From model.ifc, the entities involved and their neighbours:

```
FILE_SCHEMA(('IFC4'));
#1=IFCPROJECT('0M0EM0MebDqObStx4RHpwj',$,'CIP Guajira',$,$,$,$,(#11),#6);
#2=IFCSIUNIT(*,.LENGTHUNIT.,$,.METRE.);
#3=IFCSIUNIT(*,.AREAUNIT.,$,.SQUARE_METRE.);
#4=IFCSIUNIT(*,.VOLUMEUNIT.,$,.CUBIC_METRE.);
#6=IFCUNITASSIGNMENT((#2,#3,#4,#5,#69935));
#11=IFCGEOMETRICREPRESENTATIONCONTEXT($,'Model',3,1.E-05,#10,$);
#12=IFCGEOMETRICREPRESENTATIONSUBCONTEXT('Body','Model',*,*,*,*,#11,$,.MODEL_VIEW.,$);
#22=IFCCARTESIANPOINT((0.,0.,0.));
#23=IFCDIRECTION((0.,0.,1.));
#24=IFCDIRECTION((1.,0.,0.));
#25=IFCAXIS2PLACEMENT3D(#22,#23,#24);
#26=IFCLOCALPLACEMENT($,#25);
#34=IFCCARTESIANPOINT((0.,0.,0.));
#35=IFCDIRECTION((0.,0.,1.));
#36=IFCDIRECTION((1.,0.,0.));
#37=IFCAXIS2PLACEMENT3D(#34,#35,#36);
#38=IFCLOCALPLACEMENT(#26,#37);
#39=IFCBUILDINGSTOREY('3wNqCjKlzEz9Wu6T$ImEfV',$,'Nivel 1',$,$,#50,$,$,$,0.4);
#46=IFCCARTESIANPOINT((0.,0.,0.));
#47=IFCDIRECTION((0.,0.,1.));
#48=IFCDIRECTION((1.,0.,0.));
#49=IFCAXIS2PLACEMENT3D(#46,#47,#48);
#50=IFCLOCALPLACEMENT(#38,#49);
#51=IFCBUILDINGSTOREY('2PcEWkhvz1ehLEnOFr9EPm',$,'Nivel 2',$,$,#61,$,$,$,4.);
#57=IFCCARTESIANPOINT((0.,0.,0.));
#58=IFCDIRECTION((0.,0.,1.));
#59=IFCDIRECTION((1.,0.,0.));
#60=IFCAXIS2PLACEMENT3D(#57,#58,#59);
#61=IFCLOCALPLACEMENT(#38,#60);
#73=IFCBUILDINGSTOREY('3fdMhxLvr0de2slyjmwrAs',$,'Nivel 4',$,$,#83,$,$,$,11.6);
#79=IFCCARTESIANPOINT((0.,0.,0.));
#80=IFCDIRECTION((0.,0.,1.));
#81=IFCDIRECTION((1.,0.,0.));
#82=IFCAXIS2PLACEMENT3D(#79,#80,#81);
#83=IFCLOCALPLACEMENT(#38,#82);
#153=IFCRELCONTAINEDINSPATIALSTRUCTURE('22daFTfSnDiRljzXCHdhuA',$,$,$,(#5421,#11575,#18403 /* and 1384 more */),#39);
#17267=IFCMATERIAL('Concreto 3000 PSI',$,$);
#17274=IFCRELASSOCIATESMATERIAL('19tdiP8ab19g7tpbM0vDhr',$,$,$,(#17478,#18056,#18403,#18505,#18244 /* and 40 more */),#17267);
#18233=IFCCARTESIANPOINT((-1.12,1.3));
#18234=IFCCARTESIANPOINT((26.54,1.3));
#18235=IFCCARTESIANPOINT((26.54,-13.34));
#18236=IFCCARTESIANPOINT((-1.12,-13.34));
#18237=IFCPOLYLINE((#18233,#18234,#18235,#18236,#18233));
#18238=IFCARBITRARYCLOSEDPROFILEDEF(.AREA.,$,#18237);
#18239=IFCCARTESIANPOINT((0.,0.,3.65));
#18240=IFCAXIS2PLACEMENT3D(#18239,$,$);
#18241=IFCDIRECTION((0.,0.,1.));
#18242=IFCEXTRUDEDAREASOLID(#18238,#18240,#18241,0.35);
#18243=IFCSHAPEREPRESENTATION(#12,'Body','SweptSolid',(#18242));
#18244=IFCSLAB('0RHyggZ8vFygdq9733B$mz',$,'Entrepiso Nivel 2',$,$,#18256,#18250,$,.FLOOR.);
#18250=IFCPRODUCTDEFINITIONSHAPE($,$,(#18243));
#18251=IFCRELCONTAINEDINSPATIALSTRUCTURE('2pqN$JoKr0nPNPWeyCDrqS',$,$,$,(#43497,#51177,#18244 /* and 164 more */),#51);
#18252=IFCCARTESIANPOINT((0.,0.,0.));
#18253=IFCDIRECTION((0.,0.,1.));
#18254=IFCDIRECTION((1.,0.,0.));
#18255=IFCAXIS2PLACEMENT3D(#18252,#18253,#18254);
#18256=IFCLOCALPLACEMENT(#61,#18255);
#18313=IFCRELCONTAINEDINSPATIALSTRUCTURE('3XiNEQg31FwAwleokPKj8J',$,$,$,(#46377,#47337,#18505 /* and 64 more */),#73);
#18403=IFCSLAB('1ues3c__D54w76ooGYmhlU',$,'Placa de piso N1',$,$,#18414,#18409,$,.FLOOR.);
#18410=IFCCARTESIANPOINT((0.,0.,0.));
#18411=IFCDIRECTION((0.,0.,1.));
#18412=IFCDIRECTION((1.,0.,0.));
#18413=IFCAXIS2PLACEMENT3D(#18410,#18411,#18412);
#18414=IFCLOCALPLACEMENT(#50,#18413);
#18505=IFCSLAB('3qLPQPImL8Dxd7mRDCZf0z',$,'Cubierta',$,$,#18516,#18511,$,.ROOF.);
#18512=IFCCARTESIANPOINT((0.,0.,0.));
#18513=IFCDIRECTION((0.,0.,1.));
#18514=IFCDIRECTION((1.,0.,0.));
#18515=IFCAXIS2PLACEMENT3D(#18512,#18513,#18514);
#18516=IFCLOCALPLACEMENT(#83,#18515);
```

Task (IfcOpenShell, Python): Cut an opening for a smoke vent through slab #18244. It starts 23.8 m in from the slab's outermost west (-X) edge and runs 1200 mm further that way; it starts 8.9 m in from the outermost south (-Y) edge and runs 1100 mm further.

```python
import numpy as np
import ifcopenshell
import ifcopenshell.api.feature
import ifcopenshell.api.geometry
import ifcopenshell.api.root
import ifcopenshell.geom
import ifcopenshell.util.placement
import ifcopenshell.util.representation
import ifcopenshell.util.shape
import ifcopenshell.util.unit

model = ifcopenshell.open("model.ifc")
unit_scale = ifcopenshell.util.unit.calculate_unit_scale(model)
settings = ifcopenshell.geom.settings()


def volume(element):
    """Net volume in cubic metres, openings subtracted."""
    shape = ifcopenshell.geom.create_shape(settings, element)
    return ifcopenshell.util.shape.get_volume(shape.geometry)


slab = model.by_id(18244)
before = volume(slab)

# Extent in the slab's own axes, in metres. The edges named are its -X and -Y sides.
slab_shape = ifcopenshell.geom.create_shape(settings, slab)
vertices = ifcopenshell.util.shape.get_vertices(slab_shape.geometry)
x_min, y_min, bottom = vertices.min(axis=0)
top = vertices[:, 2].max()

opening = ifcopenshell.api.root.create_entity(model, ifc_class="IfcOpeningElement", name="Smoke vent opening", predefined_type="OPENING")
context = ifcopenshell.util.representation.get_context(model, "Model", "Body", "MODEL_VIEW")
width, depth = 1.2, 1.1
outline = [(0.0, 0.0), (width, 0.0), (width, depth), (0.0, depth), (0.0, 0.0)]
# Overshoot both faces by 50 mm so the cut is clean.
shape = ifcopenshell.api.geometry.add_slab_representation(
    model, context=context, depth=top - bottom + 0.1, polyline=outline
)
ifcopenshell.api.geometry.assign_representation(model, product=opening, representation=shape)

matrix = ifcopenshell.util.placement.get_local_placement(slab.ObjectPlacement)
matrix[:, 3] = matrix @ np.append(np.array([x_min + 23.8, y_min + 8.9, bottom - 0.05]) / unit_scale, 1.0)
ifcopenshell.api.geometry.edit_object_placement(model, product=opening, matrix=matrix, is_si=False)
ifcopenshell.api.feature.add_feature(model, feature=opening, element=slab)

after = volume(slab)

print(f"slab volume {before:.3f} -> {after:.3f} m3")

model.write("model_edited.ifc")
```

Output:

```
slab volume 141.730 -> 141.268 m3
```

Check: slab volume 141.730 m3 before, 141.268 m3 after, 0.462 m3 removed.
